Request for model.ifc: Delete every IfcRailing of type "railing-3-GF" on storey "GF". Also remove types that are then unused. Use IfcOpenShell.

First a look at what the model holds.

```python
import ifcopenshell
import ifcopenshell.util.element

model = ifcopenshell.open("model.ifc")
print(model.schema)
storey = next(s for s in model.by_type("IfcBuildingStorey") if s.Name == "GF")
railings = [e for e in ifcopenshell.util.element.get_decomposition(storey) if e.is_a("IfcRailing")]
seen = {}
for e in railings:
    element_type = ifcopenshell.util.element.get_type(e)
    name = element_type.Name if element_type not in (None, e) else None
    seen[name] = seen.get(name, 0) + 1
for name, count in sorted(seen.items(), key=str):
    print(count, "x", name)
```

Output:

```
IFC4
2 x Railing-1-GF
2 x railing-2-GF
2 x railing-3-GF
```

```python
import ifcopenshell
import ifcopenshell.api.root
import ifcopenshell.util.element

model = ifcopenshell.open("model.ifc")

storey = next(s for s in model.by_type("IfcBuildingStorey") if s.Name == "GF")
railings = [e for e in ifcopenshell.util.element.get_decomposition(storey) if e.is_a("IfcRailing")]
targets = [e for e in railings if (t := ifcopenshell.util.element.get_type(e)) not in (None, e) and t.Name == "railing-3-GF"]
types = {ifcopenshell.util.element.get_type(e) for e in targets} - {None, *targets}

for e in targets:
    ifcopenshell.api.root.remove_product(model, product=e)
print(len(targets), "removed")

unused = [t for t in types if not ifcopenshell.util.element.get_types(t)]
for t in unused:
    ifcopenshell.api.root.remove_product(model, product=t)
print(len(unused), "unused types removed")

model.write("model_v2.ifc")
```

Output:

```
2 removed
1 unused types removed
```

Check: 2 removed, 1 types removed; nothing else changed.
